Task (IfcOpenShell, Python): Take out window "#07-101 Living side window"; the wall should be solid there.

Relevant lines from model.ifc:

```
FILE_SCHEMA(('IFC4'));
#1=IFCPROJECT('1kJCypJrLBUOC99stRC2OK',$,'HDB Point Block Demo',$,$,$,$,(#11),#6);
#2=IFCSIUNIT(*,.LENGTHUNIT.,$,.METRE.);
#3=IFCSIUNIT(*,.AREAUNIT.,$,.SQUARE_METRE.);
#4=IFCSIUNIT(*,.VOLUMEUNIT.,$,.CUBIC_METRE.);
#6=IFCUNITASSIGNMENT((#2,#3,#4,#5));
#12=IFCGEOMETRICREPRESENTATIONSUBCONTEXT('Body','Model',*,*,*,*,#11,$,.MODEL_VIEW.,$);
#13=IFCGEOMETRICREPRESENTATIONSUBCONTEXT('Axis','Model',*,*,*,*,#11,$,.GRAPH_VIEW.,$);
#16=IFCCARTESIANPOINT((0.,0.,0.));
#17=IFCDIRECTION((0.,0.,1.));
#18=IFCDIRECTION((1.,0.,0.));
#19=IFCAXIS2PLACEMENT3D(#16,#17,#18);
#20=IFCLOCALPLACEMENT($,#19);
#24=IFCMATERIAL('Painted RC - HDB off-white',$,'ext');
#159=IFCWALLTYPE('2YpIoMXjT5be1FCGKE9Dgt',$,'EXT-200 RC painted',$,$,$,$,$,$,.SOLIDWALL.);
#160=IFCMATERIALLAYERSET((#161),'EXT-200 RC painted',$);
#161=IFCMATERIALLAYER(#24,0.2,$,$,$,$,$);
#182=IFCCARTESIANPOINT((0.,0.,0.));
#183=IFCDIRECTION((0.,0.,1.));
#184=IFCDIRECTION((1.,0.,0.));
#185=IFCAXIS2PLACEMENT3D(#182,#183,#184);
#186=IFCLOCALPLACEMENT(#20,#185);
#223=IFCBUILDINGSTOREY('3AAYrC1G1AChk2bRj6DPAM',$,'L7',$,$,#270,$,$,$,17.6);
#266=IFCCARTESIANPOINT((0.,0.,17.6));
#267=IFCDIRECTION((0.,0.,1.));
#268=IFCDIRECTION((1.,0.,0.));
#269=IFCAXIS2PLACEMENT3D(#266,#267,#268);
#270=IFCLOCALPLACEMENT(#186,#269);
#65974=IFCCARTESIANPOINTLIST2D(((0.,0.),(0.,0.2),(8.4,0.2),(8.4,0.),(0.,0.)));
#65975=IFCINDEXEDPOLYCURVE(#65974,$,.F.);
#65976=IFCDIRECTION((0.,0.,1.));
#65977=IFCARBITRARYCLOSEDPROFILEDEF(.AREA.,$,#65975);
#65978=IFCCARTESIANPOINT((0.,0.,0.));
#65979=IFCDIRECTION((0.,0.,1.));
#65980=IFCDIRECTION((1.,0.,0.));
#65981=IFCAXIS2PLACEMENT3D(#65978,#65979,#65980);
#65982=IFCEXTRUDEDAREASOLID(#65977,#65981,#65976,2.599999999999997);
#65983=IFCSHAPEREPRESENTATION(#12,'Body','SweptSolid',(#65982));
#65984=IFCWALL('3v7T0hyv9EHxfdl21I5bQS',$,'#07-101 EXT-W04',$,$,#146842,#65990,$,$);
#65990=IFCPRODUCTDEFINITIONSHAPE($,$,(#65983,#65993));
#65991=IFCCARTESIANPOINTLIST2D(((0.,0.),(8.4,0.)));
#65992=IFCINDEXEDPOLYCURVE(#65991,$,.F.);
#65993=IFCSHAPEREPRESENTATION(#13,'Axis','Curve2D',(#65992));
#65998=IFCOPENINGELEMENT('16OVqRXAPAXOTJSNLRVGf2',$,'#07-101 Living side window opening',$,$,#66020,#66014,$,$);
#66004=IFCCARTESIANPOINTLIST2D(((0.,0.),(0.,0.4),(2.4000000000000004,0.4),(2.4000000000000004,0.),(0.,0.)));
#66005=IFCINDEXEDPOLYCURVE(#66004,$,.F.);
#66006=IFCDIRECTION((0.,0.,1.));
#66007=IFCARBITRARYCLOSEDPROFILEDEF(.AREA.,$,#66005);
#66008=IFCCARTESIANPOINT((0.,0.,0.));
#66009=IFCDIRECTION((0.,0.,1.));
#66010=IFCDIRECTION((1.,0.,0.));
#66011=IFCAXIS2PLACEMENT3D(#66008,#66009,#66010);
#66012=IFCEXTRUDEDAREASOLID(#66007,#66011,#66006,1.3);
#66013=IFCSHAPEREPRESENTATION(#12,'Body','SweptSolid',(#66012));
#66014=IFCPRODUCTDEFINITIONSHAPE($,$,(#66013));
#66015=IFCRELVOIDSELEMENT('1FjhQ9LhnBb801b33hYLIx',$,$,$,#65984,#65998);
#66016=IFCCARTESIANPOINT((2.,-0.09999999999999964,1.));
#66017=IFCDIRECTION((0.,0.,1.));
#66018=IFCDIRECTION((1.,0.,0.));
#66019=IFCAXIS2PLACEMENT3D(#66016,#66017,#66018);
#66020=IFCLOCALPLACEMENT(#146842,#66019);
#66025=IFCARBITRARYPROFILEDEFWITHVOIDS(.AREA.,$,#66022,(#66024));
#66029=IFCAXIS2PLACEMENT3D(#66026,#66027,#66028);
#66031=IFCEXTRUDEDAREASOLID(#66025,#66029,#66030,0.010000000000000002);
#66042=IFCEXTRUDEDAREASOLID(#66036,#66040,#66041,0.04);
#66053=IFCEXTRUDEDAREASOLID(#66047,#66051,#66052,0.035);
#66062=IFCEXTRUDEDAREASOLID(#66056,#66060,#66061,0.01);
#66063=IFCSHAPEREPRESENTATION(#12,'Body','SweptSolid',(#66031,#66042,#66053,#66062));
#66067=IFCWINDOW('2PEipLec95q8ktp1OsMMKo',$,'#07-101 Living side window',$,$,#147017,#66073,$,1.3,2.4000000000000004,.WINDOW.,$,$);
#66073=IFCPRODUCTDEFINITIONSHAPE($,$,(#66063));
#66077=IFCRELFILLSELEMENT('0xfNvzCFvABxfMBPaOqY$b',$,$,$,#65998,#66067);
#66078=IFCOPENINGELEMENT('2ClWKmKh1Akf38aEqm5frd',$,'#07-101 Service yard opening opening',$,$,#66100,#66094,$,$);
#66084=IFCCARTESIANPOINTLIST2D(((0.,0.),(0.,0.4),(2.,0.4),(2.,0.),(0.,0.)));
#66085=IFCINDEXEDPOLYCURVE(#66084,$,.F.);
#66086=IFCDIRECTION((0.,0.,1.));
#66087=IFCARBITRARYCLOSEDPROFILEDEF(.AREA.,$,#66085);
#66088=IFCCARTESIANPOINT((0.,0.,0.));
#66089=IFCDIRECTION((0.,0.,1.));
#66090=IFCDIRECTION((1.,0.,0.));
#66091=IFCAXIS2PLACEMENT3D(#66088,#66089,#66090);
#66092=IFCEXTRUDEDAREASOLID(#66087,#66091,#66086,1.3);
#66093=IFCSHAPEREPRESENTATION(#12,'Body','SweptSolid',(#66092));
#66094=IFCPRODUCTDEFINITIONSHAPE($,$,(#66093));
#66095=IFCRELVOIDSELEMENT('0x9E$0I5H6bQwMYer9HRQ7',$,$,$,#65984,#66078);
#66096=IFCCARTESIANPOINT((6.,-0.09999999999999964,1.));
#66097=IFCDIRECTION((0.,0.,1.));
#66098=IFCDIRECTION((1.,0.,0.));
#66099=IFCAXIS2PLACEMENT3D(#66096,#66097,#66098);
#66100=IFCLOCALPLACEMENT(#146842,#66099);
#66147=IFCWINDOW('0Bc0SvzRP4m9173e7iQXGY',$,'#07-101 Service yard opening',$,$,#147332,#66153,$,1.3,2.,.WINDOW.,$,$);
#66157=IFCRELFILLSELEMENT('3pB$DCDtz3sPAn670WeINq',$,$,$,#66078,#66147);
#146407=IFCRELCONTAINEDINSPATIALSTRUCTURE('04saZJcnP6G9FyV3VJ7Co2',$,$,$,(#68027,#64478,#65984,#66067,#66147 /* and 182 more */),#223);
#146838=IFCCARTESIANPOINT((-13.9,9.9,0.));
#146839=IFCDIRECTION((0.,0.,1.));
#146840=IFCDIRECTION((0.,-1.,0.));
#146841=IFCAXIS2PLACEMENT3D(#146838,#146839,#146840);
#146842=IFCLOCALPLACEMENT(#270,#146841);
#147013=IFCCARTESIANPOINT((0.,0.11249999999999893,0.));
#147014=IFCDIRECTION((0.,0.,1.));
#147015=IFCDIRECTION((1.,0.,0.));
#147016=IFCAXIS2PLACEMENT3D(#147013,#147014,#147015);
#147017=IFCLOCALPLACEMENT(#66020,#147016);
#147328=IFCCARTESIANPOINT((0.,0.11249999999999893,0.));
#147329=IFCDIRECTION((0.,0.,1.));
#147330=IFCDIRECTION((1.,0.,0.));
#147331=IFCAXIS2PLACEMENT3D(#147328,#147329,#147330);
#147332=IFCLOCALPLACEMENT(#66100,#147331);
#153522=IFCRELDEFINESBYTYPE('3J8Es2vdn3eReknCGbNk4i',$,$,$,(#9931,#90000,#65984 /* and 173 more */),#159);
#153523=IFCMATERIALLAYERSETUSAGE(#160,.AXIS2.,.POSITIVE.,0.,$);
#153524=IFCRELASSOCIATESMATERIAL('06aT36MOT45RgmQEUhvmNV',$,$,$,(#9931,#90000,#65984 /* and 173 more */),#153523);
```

```python
import ifcopenshell
import ifcopenshell.api.feature
import ifcopenshell.api.root
import ifcopenshell.geom
import ifcopenshell.util.shape

model = ifcopenshell.open("model.ifc")
settings = ifcopenshell.geom.settings()


def volume(element):
    """Net volume in cubic metres, openings subtracted."""
    shape = ifcopenshell.geom.create_shape(settings, element)
    return ifcopenshell.util.shape.get_volume(shape.geometry)


window = model.by_guid("2PEipLec95q8ktp1OsMMKo")
opening = window.FillsVoids[0].RelatingOpeningElement
wall = opening.VoidsElements[0].RelatingBuildingElement
before = volume(wall)

ifcopenshell.api.root.remove_product(model, product=window)
ifcopenshell.api.feature.remove_feature(model, feature=opening)

after = volume(wall)

print(f"wall volume {before:.3f} -> {after:.3f} m3")

model.write("model_rev.ifc")
```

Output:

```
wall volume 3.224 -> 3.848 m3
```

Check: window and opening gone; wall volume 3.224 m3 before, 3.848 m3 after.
